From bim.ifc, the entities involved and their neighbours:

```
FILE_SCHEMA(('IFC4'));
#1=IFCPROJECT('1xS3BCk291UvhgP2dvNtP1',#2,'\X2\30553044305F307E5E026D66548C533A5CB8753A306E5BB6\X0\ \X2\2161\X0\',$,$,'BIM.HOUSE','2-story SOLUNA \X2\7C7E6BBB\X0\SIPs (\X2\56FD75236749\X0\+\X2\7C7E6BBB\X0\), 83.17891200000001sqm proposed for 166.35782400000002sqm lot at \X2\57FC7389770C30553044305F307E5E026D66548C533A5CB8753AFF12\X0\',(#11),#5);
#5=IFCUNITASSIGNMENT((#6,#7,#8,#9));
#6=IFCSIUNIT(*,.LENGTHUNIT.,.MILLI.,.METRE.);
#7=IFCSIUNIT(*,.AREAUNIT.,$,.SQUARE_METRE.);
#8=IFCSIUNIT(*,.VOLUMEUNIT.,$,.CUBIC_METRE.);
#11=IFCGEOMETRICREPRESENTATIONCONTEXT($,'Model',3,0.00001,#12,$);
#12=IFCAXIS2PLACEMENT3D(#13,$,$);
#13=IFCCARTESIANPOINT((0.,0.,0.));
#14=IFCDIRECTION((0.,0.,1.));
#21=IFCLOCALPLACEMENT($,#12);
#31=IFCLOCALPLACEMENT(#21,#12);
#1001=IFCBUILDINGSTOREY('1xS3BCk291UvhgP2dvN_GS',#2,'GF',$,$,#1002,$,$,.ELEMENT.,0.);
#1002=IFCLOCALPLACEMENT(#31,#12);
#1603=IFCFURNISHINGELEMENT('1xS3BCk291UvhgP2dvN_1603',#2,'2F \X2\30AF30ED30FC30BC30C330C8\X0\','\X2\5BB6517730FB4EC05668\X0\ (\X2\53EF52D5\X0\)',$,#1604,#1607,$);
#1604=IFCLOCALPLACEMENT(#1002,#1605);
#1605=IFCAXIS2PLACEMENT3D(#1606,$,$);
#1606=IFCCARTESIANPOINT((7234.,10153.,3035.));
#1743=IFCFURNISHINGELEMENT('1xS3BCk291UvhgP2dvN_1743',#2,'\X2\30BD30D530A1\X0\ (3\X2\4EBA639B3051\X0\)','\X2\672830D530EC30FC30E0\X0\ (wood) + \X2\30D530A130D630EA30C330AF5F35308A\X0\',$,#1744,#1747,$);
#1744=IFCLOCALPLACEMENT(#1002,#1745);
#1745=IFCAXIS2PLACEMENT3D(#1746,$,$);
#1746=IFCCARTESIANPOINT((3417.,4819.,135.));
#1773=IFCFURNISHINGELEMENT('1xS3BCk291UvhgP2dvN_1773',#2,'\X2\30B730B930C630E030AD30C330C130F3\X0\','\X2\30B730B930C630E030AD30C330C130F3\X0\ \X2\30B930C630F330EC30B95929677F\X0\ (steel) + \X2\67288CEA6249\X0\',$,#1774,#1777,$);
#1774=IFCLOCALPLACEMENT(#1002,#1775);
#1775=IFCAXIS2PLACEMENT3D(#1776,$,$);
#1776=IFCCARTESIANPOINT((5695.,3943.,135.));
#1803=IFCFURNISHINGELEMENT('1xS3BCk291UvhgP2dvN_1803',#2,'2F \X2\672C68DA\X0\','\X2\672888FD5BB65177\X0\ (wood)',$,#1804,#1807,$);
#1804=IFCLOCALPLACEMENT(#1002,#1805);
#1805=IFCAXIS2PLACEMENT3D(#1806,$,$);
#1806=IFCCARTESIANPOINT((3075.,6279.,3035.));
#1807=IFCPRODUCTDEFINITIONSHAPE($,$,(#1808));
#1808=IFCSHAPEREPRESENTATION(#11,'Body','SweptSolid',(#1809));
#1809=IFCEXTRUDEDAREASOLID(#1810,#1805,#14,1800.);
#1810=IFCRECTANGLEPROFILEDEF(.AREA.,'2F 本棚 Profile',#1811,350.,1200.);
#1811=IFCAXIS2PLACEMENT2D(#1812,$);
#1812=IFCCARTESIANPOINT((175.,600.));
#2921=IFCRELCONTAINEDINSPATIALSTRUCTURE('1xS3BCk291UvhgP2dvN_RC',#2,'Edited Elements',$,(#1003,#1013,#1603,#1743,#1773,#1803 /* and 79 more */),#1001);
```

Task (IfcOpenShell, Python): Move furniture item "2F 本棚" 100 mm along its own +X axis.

```python
import ifcopenshell
import ifcopenshell.api.geometry
import ifcopenshell.util.placement

model = ifcopenshell.open("bim.ifc")

item = model.by_guid("1xS3BCk291UvhgP2dvN_1803")
matrix = ifcopenshell.util.placement.get_local_placement(item.ObjectPlacement)
matrix[:3, 3] += matrix[:3, 0] * 100.0
ifcopenshell.api.geometry.edit_object_placement(model, product=item, matrix=matrix, is_si=False)

print(ifcopenshell.util.placement.get_local_placement(item.ObjectPlacement).round(3) + 0.0)

model.write("bim_edited.ifc")
```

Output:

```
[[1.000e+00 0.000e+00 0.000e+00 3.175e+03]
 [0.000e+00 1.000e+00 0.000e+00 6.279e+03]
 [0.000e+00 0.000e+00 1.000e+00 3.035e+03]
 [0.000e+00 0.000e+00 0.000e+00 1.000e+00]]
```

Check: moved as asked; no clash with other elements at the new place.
